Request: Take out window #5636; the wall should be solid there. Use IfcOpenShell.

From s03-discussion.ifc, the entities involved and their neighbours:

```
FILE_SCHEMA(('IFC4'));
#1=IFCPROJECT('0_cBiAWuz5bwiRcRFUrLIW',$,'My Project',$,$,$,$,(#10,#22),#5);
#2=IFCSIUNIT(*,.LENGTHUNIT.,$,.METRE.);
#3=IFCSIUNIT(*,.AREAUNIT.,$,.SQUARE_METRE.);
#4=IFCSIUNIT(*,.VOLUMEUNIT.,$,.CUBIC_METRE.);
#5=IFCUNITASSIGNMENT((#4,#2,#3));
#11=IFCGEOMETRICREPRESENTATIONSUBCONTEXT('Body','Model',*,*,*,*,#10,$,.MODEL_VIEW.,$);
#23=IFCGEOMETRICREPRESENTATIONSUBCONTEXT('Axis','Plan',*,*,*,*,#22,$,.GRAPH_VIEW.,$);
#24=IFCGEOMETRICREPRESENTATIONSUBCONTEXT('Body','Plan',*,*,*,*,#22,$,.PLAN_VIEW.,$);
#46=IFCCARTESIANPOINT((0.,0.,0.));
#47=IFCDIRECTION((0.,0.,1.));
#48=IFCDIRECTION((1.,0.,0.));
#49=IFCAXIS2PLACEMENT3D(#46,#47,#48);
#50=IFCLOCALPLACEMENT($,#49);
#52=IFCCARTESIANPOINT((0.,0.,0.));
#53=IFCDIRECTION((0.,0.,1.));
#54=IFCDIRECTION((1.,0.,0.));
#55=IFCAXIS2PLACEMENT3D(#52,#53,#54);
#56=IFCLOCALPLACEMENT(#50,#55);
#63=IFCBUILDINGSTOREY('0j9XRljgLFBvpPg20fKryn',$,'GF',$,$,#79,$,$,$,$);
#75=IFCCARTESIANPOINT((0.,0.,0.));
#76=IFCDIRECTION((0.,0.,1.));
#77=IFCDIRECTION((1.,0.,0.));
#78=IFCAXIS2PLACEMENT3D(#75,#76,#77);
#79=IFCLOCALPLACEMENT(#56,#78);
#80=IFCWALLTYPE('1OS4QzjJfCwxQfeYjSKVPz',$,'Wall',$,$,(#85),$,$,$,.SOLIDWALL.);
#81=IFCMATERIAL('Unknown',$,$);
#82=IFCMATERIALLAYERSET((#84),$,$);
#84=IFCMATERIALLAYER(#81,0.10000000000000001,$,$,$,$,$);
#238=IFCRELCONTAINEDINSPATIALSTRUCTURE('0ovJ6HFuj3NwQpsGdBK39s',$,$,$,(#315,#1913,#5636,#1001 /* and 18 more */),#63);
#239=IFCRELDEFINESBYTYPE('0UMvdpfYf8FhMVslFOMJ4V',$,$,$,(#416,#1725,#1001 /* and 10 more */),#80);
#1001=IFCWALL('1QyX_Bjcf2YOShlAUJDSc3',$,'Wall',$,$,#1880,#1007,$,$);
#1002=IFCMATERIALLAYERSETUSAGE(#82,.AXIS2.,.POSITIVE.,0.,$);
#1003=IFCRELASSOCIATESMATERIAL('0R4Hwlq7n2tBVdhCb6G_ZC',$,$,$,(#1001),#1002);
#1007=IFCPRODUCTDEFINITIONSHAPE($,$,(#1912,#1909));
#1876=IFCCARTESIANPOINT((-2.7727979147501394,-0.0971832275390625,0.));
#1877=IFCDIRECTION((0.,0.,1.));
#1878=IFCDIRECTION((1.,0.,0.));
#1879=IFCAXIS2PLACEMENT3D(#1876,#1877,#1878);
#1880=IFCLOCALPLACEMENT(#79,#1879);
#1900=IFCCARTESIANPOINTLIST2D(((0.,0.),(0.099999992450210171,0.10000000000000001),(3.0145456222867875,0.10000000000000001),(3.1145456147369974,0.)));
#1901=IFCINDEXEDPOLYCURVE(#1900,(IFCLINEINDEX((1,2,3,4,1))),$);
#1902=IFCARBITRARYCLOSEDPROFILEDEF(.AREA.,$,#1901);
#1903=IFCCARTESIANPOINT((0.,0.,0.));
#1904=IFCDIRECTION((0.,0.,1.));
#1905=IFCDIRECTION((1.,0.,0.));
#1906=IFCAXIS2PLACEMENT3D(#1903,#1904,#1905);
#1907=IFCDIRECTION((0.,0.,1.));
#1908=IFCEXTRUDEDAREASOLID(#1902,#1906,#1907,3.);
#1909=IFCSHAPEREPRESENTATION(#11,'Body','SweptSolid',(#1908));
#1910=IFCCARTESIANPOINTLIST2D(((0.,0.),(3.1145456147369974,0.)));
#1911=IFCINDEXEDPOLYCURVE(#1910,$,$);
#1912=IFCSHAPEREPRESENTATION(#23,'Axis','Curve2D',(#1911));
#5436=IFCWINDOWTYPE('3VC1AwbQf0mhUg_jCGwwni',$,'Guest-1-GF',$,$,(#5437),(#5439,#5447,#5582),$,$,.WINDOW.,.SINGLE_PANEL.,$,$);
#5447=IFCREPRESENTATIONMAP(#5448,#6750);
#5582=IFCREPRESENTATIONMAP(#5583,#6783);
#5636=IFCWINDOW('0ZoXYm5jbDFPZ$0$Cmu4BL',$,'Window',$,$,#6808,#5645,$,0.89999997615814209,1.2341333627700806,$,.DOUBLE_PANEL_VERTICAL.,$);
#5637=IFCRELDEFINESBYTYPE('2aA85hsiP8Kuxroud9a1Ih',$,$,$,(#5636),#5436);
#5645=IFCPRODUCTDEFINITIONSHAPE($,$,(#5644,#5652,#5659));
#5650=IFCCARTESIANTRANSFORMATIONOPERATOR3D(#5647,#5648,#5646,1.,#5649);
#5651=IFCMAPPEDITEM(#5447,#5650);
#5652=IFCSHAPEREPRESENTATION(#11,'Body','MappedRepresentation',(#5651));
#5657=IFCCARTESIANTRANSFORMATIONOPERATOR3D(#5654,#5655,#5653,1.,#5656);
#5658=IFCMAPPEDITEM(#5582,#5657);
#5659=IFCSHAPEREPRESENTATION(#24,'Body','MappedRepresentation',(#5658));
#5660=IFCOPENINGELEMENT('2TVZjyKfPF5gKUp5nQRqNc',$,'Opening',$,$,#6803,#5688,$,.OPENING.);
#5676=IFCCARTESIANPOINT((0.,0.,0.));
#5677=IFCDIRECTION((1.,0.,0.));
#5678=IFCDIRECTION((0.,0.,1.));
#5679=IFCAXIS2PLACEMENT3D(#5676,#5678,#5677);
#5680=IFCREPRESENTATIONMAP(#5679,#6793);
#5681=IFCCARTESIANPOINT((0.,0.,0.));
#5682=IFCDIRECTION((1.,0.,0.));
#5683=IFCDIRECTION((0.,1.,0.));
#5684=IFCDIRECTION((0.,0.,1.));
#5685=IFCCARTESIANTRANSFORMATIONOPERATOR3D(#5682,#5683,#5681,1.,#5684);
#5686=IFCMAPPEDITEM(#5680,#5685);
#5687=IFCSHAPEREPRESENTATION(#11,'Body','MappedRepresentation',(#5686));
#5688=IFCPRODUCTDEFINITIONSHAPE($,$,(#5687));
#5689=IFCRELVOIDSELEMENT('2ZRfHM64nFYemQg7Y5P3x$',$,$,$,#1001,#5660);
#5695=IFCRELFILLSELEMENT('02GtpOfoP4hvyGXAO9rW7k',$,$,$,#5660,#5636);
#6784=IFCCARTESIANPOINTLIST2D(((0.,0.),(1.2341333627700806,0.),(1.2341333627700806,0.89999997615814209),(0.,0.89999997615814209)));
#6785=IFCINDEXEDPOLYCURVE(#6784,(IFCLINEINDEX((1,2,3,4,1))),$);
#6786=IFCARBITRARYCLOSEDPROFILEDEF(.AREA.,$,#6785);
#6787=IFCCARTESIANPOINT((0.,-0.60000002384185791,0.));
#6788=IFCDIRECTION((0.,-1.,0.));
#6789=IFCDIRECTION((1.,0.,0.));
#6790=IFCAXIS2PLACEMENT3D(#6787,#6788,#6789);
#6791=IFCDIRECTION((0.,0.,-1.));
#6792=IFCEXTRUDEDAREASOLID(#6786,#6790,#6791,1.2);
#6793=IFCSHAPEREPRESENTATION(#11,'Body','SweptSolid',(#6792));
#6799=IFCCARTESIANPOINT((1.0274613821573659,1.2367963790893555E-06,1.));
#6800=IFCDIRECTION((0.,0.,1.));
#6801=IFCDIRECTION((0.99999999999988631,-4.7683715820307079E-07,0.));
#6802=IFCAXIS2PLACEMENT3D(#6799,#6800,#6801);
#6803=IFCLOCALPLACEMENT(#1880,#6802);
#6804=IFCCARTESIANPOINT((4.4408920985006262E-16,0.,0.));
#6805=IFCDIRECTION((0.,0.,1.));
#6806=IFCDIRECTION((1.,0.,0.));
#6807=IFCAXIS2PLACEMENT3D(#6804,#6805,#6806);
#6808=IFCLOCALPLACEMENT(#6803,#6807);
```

```python
import ifcopenshell
import ifcopenshell.api.feature
import ifcopenshell.api.root
import ifcopenshell.geom
import ifcopenshell.util.shape

model = ifcopenshell.open("s03-discussion.ifc")
settings = ifcopenshell.geom.settings()


def volume(element):
    """Net volume in cubic metres, openings subtracted."""
    shape = ifcopenshell.geom.create_shape(settings, element)
    return ifcopenshell.util.shape.get_volume(shape.geometry)


window = model.by_guid("0ZoXYm5jbDFPZ$0$Cmu4BL")
opening = window.FillsVoids[0].RelatingOpeningElement
wall = opening.VoidsElements[0].RelatingBuildingElement
before = volume(wall)

ifcopenshell.api.root.remove_product(model, product=window)
ifcopenshell.api.feature.remove_feature(model, feature=opening)

after = volume(wall)

print(f"wall volume {before:.3f} -> {after:.3f} m3")

model.write("s03-discussion_edited.ifc")
```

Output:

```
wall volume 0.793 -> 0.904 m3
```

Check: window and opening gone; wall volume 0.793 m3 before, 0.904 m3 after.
